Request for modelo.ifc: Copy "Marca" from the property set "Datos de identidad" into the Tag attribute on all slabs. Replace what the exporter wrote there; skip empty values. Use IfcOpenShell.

First a look at what the model holds.

```python
import ifcopenshell
import ifcopenshell.util.element

model = ifcopenshell.open("modelo.ifc")
print(model.schema)
slabs = model.by_type("IfcSlab")
print(len(slabs), "slabs")
for e in slabs[:8]:
    source = ifcopenshell.util.element.get_pset(e, "Datos de identidad", "Marca")
    target = e.Tag
    print(e.id(), repr(source), repr(target), sep=" | ")
```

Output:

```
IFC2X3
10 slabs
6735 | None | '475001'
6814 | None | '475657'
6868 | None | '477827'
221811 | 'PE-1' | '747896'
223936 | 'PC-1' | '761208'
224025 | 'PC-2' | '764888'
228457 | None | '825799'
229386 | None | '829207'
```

```python
import ifcopenshell
import ifcopenshell.util.element

model = ifcopenshell.open("modelo.ifc")

count = 0
for e in model.by_type("IfcSlab"):
    value = ifcopenshell.util.element.get_pset(e, "Datos de identidad", "Marca")
    current = e.Tag
    if not value or not value.strip() or current == value:
        continue
    e.Tag = value
    count += 1

print(count, "slabs updated")

model.write("modelo-out.ifc")
```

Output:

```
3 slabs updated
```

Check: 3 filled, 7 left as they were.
